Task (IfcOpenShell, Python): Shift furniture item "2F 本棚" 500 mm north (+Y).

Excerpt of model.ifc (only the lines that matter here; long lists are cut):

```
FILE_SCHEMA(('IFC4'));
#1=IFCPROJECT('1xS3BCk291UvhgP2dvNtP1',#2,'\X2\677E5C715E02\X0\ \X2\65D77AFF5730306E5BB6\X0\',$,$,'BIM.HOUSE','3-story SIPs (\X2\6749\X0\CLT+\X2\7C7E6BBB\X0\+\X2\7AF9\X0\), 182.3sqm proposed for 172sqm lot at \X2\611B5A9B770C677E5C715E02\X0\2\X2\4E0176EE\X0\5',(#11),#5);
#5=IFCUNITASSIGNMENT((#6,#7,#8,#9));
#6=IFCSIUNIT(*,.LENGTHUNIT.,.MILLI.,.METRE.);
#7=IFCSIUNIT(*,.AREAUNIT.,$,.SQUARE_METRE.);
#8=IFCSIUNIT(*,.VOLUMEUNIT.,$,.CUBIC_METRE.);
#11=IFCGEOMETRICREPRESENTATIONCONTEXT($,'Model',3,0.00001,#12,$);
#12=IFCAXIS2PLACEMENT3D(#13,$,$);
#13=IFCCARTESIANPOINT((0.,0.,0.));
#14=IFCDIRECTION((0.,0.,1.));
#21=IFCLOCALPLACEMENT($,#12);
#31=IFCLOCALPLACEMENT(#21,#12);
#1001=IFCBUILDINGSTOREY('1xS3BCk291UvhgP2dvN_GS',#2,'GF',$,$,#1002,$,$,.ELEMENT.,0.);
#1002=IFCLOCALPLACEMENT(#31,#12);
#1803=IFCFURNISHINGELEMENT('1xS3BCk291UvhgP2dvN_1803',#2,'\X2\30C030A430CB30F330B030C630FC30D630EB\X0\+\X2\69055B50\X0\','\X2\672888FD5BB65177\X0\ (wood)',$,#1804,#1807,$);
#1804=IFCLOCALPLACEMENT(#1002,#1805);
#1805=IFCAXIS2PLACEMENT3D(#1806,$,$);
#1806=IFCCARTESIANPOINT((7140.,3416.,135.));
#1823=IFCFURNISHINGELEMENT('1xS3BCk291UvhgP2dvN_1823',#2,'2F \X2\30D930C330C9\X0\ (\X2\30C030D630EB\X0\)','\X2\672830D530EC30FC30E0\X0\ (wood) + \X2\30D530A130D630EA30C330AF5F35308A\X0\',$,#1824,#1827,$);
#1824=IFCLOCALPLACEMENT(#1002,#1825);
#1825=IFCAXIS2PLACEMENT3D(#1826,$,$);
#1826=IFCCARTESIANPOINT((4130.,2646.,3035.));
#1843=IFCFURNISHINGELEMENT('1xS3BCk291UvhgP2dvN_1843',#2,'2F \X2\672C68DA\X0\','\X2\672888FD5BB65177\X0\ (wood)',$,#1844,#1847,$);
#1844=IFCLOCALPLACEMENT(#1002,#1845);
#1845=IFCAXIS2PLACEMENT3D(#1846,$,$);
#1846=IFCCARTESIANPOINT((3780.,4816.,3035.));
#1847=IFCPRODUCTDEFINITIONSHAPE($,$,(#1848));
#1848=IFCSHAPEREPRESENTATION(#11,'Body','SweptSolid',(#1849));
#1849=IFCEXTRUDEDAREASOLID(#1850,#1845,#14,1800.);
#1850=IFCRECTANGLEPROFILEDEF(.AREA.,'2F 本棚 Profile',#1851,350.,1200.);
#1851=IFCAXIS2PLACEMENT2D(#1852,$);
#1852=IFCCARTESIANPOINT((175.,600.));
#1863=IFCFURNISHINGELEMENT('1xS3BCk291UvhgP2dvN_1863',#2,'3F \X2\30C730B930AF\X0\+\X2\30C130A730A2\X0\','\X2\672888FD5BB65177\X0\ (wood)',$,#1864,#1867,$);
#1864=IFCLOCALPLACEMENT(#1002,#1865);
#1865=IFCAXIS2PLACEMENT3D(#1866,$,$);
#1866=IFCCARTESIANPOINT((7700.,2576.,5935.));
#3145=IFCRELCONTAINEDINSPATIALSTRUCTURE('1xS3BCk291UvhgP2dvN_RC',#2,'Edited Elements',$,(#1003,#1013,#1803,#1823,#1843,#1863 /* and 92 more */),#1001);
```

```python
import ifcopenshell
import ifcopenshell.api.geometry
import ifcopenshell.util.placement
import ifcopenshell.util.unit

model = ifcopenshell.open("model.ifc")
unit_scale = ifcopenshell.util.unit.calculate_unit_scale(model)

item = model.by_id(1843)
matrix = ifcopenshell.util.placement.get_local_placement(item.ObjectPlacement)
matrix[1, 3] += 0.5 / unit_scale
ifcopenshell.api.geometry.edit_object_placement(model, product=item, matrix=matrix, is_si=False)

print(ifcopenshell.util.placement.get_local_placement(item.ObjectPlacement).round(3) + 0.0)

model.write("model_updated.ifc")
```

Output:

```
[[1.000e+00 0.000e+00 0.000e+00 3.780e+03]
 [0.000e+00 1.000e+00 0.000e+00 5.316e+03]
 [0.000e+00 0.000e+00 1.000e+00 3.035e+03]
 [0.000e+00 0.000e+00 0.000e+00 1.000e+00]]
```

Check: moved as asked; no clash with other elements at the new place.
